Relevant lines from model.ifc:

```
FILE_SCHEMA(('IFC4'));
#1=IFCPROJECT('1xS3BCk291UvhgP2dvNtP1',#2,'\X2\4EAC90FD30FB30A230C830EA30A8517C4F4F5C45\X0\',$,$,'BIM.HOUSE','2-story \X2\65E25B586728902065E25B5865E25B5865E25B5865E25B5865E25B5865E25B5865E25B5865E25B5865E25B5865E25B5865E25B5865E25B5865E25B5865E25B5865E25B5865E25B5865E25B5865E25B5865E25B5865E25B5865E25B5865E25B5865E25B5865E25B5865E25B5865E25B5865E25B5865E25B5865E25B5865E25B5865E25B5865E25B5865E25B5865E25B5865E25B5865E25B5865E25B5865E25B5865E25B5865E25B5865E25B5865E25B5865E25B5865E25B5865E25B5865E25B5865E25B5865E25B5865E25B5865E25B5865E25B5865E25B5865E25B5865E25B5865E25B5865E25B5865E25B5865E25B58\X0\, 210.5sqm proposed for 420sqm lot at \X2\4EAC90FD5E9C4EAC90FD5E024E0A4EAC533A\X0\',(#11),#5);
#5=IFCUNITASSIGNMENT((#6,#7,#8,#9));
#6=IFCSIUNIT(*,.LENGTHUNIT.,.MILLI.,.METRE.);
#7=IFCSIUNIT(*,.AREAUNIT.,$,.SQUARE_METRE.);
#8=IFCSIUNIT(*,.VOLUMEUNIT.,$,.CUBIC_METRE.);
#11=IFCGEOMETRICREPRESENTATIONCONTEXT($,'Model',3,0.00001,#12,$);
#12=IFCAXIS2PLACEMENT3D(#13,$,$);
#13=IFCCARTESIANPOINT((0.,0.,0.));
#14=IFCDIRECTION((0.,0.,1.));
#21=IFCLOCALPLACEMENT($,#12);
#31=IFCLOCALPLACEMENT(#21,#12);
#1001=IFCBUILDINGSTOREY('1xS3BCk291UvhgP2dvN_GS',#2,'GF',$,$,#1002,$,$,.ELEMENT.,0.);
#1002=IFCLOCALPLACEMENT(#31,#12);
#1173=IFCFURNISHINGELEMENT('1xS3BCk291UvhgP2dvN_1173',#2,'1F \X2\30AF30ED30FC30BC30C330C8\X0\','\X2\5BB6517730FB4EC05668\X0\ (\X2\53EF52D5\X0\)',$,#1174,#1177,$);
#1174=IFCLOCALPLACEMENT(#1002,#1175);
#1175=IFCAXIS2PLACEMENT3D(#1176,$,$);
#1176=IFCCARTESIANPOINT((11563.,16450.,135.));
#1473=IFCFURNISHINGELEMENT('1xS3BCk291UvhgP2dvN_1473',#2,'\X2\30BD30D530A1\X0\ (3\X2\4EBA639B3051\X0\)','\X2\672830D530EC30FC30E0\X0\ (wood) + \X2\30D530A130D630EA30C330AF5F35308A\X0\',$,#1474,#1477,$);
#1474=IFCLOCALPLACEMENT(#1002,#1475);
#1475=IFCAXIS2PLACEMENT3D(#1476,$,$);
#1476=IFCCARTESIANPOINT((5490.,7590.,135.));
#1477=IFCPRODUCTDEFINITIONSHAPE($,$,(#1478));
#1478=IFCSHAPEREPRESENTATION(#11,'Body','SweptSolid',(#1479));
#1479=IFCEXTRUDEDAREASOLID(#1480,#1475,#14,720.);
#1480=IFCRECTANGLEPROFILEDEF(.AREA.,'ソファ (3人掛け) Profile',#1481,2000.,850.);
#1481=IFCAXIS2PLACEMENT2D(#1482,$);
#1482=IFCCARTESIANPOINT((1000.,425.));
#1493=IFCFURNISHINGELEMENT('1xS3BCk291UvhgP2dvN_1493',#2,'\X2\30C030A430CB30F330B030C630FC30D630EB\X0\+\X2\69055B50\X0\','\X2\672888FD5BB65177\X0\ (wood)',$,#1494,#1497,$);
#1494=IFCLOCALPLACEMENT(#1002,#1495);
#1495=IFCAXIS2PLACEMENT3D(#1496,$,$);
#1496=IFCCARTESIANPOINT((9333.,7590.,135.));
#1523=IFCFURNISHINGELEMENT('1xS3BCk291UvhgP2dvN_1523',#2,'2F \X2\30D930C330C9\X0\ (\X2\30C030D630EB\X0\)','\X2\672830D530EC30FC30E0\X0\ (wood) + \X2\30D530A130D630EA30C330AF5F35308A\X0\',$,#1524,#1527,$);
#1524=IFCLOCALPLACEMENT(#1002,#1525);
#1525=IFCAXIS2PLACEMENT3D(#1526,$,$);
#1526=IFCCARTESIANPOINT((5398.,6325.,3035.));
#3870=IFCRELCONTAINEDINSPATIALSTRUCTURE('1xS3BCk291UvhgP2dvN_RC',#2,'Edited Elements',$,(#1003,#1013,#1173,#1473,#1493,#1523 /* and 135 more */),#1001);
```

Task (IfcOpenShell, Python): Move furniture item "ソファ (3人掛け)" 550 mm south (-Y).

```python
import ifcopenshell
import ifcopenshell.api.geometry
import ifcopenshell.util.placement

model = ifcopenshell.open("model.ifc")

item = model.by_id(1473)
matrix = ifcopenshell.util.placement.get_local_placement(item.ObjectPlacement)
matrix[1, 3] -= 550.0
ifcopenshell.api.geometry.edit_object_placement(model, product=item, matrix=matrix, is_si=False)

print(ifcopenshell.util.placement.get_local_placement(item.ObjectPlacement).round(3) + 0.0)

model.write("model_edited.ifc")
```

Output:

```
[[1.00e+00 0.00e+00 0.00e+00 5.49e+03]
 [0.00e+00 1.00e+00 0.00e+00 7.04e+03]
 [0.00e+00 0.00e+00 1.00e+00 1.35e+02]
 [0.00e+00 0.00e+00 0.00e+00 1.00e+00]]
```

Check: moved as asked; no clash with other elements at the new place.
